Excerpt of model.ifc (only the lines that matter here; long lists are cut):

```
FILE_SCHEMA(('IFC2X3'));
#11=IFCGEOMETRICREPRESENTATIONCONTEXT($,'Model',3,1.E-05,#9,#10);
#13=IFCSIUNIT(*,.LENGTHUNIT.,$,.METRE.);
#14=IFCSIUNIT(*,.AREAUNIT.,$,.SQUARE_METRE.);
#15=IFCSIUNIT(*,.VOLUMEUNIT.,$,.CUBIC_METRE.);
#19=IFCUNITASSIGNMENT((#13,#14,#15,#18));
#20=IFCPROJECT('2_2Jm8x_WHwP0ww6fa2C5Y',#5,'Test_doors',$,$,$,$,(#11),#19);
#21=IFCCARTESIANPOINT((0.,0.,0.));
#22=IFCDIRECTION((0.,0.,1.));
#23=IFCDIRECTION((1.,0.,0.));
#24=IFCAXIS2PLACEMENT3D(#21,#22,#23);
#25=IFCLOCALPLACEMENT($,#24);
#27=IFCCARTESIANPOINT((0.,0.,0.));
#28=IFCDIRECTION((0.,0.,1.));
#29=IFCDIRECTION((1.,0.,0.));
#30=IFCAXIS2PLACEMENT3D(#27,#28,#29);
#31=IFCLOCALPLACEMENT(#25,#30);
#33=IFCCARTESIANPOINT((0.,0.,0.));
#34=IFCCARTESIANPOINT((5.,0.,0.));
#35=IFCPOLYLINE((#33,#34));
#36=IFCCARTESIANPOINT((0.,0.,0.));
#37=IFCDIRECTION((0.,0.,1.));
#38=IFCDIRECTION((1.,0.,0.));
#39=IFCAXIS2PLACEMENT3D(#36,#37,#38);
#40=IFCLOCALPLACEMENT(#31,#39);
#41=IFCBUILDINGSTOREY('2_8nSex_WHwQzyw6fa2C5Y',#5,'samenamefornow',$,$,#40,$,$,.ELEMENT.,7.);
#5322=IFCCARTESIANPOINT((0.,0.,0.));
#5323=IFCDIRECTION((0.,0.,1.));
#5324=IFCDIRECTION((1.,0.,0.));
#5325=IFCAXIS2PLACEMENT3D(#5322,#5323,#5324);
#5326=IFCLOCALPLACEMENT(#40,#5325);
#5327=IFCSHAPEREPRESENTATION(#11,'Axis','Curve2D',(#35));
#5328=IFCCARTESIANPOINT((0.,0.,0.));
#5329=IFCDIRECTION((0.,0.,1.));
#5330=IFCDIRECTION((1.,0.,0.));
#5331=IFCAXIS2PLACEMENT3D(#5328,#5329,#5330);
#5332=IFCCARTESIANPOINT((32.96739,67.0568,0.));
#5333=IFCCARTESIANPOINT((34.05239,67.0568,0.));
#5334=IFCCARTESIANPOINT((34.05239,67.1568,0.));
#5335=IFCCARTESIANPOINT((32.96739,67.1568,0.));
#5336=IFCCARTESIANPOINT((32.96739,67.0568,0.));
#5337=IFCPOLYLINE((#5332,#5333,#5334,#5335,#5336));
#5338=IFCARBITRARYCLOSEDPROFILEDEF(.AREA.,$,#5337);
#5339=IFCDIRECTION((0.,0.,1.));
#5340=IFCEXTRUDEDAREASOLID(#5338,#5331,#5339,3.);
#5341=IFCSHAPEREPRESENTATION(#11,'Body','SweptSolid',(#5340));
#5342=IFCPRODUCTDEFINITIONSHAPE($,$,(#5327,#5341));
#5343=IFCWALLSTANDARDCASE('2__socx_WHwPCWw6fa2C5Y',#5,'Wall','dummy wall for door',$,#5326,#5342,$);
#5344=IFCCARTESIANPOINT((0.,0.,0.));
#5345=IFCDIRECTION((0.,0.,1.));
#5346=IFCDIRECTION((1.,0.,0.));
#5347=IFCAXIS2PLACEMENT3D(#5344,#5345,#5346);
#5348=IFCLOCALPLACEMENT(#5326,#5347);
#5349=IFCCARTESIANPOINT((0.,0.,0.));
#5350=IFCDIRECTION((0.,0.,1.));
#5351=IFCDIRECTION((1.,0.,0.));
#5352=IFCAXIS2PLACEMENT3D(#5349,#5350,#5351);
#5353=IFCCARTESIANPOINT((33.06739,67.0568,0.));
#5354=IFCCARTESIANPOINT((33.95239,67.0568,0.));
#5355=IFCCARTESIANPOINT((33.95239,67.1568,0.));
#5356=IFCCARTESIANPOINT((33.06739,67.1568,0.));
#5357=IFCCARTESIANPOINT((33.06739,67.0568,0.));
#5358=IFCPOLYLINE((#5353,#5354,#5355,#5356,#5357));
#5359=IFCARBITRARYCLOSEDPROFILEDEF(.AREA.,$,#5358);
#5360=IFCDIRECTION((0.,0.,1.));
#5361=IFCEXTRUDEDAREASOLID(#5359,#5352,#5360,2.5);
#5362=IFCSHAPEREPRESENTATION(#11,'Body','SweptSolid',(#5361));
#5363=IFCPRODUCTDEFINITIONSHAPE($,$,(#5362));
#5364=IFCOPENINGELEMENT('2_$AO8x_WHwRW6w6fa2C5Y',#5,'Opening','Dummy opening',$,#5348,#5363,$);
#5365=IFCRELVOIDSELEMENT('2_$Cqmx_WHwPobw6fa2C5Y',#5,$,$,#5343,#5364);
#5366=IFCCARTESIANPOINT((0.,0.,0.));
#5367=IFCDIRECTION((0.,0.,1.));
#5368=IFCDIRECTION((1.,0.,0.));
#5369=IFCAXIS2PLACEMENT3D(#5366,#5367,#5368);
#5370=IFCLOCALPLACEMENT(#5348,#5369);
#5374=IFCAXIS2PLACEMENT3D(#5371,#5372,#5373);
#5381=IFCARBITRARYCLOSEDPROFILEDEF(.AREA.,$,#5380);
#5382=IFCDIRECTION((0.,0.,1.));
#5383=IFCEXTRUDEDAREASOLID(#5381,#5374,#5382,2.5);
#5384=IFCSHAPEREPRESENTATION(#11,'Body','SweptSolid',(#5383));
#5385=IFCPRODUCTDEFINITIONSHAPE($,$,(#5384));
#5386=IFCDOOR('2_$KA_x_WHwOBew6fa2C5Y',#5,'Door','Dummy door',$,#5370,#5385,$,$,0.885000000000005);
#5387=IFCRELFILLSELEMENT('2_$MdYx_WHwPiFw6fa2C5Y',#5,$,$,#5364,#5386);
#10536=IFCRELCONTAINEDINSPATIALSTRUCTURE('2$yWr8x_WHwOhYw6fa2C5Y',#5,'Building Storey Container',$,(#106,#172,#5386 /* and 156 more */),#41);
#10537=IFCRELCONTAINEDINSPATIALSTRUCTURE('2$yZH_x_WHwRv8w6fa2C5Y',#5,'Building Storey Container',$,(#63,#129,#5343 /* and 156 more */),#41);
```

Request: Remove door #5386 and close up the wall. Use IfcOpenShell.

```python
import ifcopenshell
import ifcopenshell.api.feature
import ifcopenshell.api.root
import ifcopenshell.geom
import ifcopenshell.util.shape

model = ifcopenshell.open("model.ifc")
settings = ifcopenshell.geom.settings()


def volume(element):
    """Net volume in cubic metres, openings subtracted."""
    shape = ifcopenshell.geom.create_shape(settings, element)
    return ifcopenshell.util.shape.get_volume(shape.geometry)


door = model.by_guid("2_$KA_x_WHwOBew6fa2C5Y")
opening = door.FillsVoids[0].RelatingOpeningElement
wall = opening.VoidsElements[0].RelatingBuildingElement
before = volume(wall)

ifcopenshell.api.root.remove_product(model, product=door)
ifcopenshell.api.feature.remove_feature(model, feature=opening)

after = volume(wall)

print(f"wall volume {before:.3f} -> {after:.3f} m3")

model.write("model-out.ifc")
```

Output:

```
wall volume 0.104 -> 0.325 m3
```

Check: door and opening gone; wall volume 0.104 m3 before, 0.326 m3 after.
